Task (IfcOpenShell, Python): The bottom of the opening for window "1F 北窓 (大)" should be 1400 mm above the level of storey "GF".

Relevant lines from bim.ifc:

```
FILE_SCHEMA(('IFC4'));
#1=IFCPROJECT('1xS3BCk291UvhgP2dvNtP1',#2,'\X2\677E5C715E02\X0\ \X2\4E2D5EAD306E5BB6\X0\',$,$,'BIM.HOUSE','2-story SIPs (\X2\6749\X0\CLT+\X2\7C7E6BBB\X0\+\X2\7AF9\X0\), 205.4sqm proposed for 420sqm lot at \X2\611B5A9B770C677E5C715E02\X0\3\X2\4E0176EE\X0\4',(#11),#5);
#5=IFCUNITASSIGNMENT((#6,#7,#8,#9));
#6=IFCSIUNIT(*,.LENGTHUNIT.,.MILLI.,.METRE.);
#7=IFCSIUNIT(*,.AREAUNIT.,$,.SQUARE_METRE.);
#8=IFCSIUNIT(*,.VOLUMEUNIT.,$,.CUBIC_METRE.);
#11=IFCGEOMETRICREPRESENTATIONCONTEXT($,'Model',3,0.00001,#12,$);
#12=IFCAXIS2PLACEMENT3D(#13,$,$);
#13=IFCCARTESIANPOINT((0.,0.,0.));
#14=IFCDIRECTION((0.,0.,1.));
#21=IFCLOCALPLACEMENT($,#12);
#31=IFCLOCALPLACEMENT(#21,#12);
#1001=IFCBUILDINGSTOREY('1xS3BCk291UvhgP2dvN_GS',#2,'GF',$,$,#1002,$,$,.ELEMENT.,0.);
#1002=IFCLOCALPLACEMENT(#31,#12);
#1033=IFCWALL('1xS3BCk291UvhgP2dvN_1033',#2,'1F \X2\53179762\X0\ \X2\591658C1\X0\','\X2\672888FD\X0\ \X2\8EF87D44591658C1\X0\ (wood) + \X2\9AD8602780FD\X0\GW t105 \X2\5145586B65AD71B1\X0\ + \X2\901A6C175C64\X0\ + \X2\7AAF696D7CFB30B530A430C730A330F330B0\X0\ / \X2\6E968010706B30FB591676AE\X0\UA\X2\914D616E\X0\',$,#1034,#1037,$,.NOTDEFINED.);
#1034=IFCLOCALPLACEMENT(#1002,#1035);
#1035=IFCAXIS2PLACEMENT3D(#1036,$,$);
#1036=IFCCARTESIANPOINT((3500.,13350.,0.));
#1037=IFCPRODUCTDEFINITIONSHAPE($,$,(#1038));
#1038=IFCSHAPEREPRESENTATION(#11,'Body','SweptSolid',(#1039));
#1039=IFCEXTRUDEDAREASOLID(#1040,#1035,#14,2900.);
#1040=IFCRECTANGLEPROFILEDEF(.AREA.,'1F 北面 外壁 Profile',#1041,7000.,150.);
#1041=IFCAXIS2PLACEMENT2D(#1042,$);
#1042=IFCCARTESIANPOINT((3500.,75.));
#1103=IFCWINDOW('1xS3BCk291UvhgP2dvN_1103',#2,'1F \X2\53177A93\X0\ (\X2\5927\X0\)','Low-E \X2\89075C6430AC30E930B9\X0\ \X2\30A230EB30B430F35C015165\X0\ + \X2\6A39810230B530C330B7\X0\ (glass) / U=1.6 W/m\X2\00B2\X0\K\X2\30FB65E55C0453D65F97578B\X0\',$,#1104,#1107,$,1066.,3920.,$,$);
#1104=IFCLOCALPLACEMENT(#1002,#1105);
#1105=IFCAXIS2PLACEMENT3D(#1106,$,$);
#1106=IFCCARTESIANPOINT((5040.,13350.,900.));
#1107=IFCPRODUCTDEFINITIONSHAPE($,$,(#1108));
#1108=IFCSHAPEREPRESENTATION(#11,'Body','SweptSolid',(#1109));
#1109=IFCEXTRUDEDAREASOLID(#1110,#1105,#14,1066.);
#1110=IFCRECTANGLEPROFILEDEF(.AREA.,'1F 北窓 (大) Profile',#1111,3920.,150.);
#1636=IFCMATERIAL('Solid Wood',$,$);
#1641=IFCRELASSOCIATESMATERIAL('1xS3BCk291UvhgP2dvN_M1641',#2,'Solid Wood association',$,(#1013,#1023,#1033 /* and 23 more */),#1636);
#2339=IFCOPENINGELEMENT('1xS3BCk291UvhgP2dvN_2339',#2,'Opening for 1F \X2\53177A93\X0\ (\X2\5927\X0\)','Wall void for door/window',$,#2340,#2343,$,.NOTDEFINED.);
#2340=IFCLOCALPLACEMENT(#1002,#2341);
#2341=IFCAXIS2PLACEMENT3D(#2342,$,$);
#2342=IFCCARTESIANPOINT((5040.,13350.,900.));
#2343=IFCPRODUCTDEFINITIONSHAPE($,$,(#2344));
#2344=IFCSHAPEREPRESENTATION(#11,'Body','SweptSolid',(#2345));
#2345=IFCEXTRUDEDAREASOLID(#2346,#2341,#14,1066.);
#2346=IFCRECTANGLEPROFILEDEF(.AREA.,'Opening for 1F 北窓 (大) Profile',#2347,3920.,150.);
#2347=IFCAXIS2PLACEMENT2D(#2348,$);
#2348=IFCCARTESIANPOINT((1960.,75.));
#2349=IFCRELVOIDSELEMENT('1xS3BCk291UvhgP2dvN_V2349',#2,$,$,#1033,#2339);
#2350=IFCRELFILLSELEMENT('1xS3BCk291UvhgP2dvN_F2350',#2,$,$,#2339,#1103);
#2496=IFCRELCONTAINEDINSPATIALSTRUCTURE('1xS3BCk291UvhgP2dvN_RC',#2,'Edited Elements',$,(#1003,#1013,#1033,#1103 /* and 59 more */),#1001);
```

```python
import numpy as np
import ifcopenshell
import ifcopenshell.api.geometry
import ifcopenshell.geom
import ifcopenshell.util.element
import ifcopenshell.util.placement
import ifcopenshell.util.shape
import ifcopenshell.util.unit

model = ifcopenshell.open("bim.ifc")
unit_scale = ifcopenshell.util.unit.calculate_unit_scale(model)

window = model.by_id(1103)
opening = window.FillsVoids[0].RelatingOpeningElement
storey = ifcopenshell.util.element.get_container(window, ifc_class="IfcBuildingStorey")
level = ifcopenshell.util.placement.get_local_placement(storey.ObjectPlacement)[2, 3]

# The opening's origin need not be at the sill, so measure its lowest point.
shape = ifcopenshell.geom.create_shape(ifcopenshell.geom.settings(), opening)
bottom = ifcopenshell.util.shape.get_shape_bottom_elevation(shape, shape.geometry) / unit_scale
dz = level + 1400.0 - bottom

shift = np.array([0.0, 0.0, dz])
# The window is not placed relative to its opening, so move both.
for product in (opening, window):
    matrix = ifcopenshell.util.placement.get_local_placement(product.ObjectPlacement)
    matrix[:3, 3] += shift
    ifcopenshell.api.geometry.edit_object_placement(model, product=product, matrix=matrix, is_si=False)

print(f"moved by {dz * unit_scale:+.3f} m")

model.write("bim_updated.ifc")
```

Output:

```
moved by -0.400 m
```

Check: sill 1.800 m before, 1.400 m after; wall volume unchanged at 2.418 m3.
